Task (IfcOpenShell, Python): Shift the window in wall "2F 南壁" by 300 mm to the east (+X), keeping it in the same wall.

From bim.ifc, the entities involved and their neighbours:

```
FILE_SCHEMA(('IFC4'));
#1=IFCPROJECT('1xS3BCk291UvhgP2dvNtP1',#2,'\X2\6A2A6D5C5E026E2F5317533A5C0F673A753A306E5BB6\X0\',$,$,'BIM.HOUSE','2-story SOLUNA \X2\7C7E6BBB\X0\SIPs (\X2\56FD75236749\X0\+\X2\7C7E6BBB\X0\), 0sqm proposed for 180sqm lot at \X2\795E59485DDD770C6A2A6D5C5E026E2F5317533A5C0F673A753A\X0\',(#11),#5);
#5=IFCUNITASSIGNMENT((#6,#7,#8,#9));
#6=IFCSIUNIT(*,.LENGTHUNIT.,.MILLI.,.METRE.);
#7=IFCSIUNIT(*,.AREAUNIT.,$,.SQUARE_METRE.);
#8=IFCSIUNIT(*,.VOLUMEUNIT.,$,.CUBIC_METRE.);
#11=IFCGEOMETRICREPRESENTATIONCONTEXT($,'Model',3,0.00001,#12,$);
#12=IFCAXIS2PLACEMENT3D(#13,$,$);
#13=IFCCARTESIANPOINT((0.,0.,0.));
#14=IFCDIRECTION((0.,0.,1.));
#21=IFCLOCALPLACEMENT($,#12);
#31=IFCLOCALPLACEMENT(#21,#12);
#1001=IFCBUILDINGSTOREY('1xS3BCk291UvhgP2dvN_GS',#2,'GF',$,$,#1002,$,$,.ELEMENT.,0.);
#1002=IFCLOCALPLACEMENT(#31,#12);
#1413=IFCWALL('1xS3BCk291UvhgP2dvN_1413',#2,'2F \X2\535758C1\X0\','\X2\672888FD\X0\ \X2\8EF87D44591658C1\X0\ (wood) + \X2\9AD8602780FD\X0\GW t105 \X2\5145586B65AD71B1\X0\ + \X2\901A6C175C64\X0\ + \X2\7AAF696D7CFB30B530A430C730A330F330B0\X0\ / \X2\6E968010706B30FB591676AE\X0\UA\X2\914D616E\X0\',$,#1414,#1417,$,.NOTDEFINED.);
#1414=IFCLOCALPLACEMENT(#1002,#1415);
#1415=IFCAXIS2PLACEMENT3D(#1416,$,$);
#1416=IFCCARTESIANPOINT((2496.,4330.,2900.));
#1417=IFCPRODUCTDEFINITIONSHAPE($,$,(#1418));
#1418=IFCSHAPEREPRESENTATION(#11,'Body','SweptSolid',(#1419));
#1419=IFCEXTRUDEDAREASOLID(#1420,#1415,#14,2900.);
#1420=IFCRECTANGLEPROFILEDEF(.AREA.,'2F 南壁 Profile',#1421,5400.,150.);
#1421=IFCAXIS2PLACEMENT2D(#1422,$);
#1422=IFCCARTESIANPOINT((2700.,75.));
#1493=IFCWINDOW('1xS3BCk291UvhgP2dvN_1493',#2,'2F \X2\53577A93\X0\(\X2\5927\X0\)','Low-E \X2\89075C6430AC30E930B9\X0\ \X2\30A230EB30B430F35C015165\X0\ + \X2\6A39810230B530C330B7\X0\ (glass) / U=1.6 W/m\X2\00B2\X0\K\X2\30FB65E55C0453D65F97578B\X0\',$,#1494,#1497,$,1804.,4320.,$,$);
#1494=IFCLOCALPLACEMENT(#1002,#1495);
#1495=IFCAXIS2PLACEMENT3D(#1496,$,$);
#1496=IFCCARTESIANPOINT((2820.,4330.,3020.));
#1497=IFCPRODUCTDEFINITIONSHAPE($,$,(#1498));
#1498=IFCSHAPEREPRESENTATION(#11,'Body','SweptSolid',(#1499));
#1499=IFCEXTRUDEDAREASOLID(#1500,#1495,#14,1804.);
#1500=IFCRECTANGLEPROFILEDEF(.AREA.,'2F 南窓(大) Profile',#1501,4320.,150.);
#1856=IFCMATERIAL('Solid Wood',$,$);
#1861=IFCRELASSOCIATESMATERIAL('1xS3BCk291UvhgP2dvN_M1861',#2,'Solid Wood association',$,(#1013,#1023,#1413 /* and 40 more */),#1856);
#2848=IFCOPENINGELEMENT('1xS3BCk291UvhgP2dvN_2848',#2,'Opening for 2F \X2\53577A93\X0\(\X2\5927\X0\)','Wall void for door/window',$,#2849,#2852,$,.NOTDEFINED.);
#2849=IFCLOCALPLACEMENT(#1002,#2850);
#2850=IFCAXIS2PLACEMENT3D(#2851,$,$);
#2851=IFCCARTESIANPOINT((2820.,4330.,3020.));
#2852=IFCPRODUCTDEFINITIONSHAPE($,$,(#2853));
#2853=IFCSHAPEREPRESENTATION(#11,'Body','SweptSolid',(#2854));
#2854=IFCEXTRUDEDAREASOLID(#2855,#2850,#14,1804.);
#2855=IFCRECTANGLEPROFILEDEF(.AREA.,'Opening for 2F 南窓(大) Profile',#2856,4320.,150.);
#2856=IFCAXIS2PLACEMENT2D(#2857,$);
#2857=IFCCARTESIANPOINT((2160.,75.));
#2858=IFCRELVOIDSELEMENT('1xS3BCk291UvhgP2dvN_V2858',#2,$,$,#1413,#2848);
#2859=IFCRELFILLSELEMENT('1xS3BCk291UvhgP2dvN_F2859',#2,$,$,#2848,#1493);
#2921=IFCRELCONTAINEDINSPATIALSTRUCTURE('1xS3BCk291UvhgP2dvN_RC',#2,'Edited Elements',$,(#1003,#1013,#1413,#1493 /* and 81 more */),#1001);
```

```python
import ifcopenshell
import ifcopenshell.api.geometry
import ifcopenshell.util.placement

model = ifcopenshell.open("bim.ifc")

window = model.by_guid("1xS3BCk291UvhgP2dvN_1493")
opening = window.FillsVoids[0].RelatingOpeningElement
wall = opening.VoidsElements[0].RelatingBuildingElement

wall_matrix = ifcopenshell.util.placement.get_local_placement(wall.ObjectPlacement)
shift = wall_matrix[:3, 0] * 300.0
before = ifcopenshell.util.placement.get_local_placement(window.ObjectPlacement)[:3, 3].copy()

# The window is not placed relative to its opening, so move both.
for product in (opening, window):
    matrix = ifcopenshell.util.placement.get_local_placement(product.ObjectPlacement)
    matrix[:3, 3] += shift
    ifcopenshell.api.geometry.edit_object_placement(model, product=product, matrix=matrix, is_si=False)

after = ifcopenshell.util.placement.get_local_placement(window.ObjectPlacement)[:3, 3]
print("window moved by", (after - before).round(3) + 0.0)

model.write("bim_edited.ifc")
```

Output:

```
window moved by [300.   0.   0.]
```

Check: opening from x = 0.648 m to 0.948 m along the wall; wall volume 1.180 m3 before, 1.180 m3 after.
